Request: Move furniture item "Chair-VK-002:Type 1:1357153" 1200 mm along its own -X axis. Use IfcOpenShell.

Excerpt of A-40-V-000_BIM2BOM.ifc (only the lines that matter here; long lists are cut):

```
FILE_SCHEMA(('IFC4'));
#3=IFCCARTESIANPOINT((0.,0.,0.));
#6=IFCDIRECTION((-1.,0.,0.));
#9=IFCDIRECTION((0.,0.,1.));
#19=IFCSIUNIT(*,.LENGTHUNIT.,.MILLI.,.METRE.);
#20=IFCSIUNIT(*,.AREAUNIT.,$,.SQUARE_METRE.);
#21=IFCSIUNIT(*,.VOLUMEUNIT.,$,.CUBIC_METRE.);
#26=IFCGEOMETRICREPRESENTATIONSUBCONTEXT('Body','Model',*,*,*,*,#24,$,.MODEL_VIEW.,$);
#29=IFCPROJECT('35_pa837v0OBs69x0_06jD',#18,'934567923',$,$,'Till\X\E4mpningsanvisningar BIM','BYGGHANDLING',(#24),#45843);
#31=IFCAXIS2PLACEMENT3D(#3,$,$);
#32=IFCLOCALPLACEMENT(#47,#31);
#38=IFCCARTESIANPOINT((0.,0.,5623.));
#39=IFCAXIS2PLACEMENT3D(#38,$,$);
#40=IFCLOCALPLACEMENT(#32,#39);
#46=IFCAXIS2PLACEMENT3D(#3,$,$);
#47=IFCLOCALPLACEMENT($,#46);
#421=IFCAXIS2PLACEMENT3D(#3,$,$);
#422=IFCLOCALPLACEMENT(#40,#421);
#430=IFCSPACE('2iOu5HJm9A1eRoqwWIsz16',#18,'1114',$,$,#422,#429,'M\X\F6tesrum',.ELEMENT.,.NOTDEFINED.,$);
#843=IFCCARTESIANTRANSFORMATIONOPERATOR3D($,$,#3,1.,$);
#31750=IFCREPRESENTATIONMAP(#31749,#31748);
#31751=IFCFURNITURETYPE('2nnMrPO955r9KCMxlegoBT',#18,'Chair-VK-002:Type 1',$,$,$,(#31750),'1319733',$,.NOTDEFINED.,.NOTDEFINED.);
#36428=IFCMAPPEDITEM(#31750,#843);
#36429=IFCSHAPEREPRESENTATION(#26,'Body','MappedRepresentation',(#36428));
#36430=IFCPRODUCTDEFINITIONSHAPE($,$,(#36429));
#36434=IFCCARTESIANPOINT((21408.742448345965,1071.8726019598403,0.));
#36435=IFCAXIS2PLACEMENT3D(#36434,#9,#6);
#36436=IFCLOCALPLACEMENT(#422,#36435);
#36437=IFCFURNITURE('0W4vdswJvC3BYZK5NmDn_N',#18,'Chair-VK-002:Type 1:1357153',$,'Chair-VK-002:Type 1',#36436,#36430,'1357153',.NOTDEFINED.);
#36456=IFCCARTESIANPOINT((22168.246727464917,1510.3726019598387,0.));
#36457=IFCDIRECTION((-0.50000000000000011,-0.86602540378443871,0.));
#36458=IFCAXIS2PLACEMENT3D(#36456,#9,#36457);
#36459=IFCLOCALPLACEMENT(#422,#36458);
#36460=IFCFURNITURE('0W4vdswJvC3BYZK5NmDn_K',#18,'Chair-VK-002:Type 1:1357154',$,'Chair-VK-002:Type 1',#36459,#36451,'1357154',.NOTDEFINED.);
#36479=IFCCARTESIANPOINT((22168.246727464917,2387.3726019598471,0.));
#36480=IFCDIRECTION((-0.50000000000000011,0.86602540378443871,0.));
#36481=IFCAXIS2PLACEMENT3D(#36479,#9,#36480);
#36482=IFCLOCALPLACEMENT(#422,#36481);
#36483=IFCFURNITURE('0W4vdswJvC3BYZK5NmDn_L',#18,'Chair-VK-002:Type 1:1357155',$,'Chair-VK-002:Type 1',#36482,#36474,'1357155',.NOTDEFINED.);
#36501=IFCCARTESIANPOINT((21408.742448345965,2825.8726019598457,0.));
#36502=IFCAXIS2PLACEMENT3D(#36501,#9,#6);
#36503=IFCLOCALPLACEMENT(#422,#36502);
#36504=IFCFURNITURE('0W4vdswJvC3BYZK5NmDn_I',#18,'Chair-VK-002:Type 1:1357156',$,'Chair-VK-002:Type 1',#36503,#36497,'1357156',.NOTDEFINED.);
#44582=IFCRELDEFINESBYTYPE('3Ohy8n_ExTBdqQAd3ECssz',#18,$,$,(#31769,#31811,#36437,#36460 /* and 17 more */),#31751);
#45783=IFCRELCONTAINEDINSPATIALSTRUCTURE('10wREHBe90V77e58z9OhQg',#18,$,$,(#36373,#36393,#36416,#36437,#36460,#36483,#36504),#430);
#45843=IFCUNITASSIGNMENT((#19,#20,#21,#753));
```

```python
import ifcopenshell
import ifcopenshell.api.geometry
import ifcopenshell.util.placement

model = ifcopenshell.open("A-40-V-000_BIM2BOM.ifc")

item = model.by_guid("0W4vdswJvC3BYZK5NmDn_N")
matrix = ifcopenshell.util.placement.get_local_placement(item.ObjectPlacement)
matrix[:3, 3] -= matrix[:3, 0] * 1200.0
ifcopenshell.api.geometry.edit_object_placement(model, product=item, matrix=matrix, is_si=False)

print(ifcopenshell.util.placement.get_local_placement(item.ObjectPlacement).round(3) + 0.0)

model.write("A-40-V-000_BIM2BOM_rev.ifc")
```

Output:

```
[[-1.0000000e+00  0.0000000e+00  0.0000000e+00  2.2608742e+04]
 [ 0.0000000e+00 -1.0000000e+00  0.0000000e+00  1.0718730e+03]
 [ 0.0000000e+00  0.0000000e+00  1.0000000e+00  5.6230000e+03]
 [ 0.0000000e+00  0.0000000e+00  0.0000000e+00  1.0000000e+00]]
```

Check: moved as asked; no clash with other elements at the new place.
